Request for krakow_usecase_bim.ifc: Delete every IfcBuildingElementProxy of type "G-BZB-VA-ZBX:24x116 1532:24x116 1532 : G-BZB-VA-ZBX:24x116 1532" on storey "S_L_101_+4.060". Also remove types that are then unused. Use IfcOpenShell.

First a look at what the model holds.

```python
import ifcopenshell
import ifcopenshell.util.element

model = ifcopenshell.open("krakow_usecase_bim.ifc")
print(model.schema)
storey = next(s for s in model.by_type("IfcBuildingStorey") if s.Name == "S_L_101_+4.060")
proxies = [e for e in ifcopenshell.util.element.get_decomposition(storey) if e.is_a("IfcBuildingElementProxy")]
seen = {}
for e in proxies:
    element_type = ifcopenshell.util.element.get_type(e)
    name = element_type.Name if element_type not in (None, e) else None
    seen[name] = seen.get(name, 0) + 1
for name, count in sorted(seen.items(), key=str):
    print(count, "x", name)
```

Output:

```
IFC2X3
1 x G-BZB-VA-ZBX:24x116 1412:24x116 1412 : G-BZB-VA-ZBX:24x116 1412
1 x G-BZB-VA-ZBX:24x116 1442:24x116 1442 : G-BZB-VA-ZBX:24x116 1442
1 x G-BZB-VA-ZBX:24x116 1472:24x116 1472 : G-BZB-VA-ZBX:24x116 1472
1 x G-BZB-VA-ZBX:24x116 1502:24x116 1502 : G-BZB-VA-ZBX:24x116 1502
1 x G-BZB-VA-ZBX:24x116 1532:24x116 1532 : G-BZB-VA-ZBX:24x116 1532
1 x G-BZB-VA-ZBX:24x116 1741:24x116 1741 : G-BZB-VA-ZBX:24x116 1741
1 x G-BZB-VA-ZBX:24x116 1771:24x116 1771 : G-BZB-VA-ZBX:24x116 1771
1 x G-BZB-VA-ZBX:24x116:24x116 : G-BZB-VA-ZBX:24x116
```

```python
import ifcopenshell
import ifcopenshell.api.root
import ifcopenshell.util.element

model = ifcopenshell.open("krakow_usecase_bim.ifc")

storey = next(s for s in model.by_type("IfcBuildingStorey") if s.Name == "S_L_101_+4.060")
proxies = [e for e in ifcopenshell.util.element.get_decomposition(storey) if e.is_a("IfcBuildingElementProxy")]
targets = [e for e in proxies if (t := ifcopenshell.util.element.get_type(e)) not in (None, e) and t.Name == "G-BZB-VA-ZBX:24x116 1532:24x116 1532 : G-BZB-VA-ZBX:24x116 1532"]
types = {ifcopenshell.util.element.get_type(e) for e in targets} - {None, *targets}

for e in targets:
    ifcopenshell.api.root.remove_product(model, product=e)
print(len(targets), "removed")

unused = [t for t in types if not ifcopenshell.util.element.get_types(t)]
for t in unused:
    ifcopenshell.api.root.remove_product(model, product=t)
print(len(unused), "unused types removed")

model.write("krakow_usecase_bim-out.ifc")
```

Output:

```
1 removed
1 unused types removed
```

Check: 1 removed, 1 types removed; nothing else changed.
